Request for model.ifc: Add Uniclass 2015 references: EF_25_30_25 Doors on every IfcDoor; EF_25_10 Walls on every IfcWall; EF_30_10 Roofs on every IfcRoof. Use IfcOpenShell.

First a look at what the model holds.

```python
import ifcopenshell

model = ifcopenshell.open("model.ifc")
print(model.schema)
print("classifications:", [c.Name for c in model.by_type("IfcClassification")])
for ifc_class in ("IfcDoor", "IfcRoof", "IfcStair", "IfcWall", "IfcWindow"):
    print(ifc_class, len(model.by_type(ifc_class)))
```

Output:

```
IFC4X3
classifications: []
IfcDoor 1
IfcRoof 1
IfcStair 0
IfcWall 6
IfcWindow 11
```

```python
import ifcopenshell
import ifcopenshell.api.classification

model = ifcopenshell.open("model.ifc")

system = ifcopenshell.api.classification.add_classification(model, classification="Uniclass 2015")

codes = {
    "IfcDoor": ("EF_25_30_25", "Doors"),
    "IfcWall": ("EF_25_10", "Walls"),
    "IfcRoof": ("EF_30_10", "Roofs"),
}
for ifc_class, (code, name) in codes.items():
    products = model.by_type(ifc_class)
    ifcopenshell.api.classification.add_reference(
        model, products=products, classification=system, identification=code, name=name
    )
    print(code, len(products))

model.write("model_v2.ifc")
```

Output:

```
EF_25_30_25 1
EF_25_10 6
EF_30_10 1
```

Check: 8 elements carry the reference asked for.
